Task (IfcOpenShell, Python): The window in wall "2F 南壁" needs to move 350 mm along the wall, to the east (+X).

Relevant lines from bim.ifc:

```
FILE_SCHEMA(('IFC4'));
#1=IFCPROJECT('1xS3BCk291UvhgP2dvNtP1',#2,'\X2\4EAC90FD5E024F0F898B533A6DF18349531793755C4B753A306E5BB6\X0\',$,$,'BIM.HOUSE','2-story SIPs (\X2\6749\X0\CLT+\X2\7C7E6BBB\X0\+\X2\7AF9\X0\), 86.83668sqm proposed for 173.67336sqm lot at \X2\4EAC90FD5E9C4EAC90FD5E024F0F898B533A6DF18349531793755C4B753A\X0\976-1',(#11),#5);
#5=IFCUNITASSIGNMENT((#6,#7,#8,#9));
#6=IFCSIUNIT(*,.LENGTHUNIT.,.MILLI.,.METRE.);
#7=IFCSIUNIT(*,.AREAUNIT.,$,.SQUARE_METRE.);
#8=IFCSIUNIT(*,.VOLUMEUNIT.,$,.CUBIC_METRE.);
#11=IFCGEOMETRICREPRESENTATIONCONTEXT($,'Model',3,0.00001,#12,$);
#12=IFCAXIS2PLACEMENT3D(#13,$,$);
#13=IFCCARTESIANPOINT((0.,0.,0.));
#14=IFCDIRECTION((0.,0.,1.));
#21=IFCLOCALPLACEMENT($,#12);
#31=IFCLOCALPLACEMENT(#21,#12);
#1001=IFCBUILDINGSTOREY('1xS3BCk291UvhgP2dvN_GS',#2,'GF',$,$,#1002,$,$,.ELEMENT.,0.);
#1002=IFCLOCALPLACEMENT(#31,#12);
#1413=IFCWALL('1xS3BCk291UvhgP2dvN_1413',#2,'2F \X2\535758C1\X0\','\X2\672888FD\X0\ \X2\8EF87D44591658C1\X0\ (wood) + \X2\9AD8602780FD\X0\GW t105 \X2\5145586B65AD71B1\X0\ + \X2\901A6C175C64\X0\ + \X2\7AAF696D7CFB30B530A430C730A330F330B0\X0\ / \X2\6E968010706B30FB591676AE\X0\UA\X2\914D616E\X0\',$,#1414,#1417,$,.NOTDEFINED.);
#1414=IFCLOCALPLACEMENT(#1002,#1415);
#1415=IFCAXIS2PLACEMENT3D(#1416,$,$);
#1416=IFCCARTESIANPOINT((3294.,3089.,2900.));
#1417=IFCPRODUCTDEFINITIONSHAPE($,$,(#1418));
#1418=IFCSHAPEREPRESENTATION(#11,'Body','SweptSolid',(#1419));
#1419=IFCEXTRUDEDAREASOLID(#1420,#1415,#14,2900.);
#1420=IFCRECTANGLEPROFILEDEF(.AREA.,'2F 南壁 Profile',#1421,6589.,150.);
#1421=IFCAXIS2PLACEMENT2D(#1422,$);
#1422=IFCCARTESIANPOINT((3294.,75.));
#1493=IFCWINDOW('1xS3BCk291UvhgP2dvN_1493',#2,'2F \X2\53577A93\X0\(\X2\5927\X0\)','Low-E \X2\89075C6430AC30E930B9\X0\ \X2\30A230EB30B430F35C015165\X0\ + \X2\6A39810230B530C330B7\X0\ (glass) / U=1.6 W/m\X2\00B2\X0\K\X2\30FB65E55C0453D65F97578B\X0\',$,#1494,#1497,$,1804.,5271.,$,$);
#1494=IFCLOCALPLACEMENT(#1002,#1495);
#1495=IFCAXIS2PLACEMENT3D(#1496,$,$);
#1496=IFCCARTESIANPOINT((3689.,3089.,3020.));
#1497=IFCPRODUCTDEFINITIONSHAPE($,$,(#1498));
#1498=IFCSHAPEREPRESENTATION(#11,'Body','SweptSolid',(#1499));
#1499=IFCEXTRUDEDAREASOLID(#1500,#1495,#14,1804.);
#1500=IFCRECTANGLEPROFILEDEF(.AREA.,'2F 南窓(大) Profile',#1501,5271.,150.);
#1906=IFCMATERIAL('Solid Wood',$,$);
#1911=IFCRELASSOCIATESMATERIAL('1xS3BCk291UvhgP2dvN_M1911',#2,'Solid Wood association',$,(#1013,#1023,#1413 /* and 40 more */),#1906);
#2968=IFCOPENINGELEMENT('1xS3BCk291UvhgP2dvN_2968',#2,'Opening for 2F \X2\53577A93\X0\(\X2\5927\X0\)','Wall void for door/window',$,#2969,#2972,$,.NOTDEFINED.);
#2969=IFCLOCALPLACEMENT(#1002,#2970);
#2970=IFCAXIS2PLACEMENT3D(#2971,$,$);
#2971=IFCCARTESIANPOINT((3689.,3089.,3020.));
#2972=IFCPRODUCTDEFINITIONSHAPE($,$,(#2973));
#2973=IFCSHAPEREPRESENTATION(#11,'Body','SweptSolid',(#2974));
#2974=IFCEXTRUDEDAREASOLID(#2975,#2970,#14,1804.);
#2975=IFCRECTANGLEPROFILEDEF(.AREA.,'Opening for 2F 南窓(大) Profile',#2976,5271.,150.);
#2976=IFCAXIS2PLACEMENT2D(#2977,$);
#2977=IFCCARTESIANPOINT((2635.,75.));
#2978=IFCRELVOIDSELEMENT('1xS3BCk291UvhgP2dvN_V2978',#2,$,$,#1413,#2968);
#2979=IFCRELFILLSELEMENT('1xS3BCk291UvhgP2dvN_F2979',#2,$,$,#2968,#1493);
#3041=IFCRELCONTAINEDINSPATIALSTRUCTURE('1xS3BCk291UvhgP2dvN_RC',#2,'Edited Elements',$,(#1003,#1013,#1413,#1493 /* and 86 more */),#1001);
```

```python
import ifcopenshell
import ifcopenshell.api.geometry
import ifcopenshell.util.placement
import ifcopenshell.util.unit

model = ifcopenshell.open("bim.ifc")
unit_scale = ifcopenshell.util.unit.calculate_unit_scale(model)

window = model.by_id(1493)
opening = window.FillsVoids[0].RelatingOpeningElement
wall = opening.VoidsElements[0].RelatingBuildingElement

wall_matrix = ifcopenshell.util.placement.get_local_placement(wall.ObjectPlacement)
shift = wall_matrix[:3, 0] * 0.35 / unit_scale
before = ifcopenshell.util.placement.get_local_placement(window.ObjectPlacement)[:3, 3].copy()

# The window is not placed relative to its opening, so move both.
for product in (opening, window):
    matrix = ifcopenshell.util.placement.get_local_placement(product.ObjectPlacement)
    matrix[:3, 3] += shift
    ifcopenshell.api.geometry.edit_object_placement(model, product=product, matrix=matrix, is_si=False)

after = ifcopenshell.util.placement.get_local_placement(window.ObjectPlacement)[:3, 3]
print("window moved by", (after - before).round(3) + 0.0)

model.write("bim_rev.ifc")
```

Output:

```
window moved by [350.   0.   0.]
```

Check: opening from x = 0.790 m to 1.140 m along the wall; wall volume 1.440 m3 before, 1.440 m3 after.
